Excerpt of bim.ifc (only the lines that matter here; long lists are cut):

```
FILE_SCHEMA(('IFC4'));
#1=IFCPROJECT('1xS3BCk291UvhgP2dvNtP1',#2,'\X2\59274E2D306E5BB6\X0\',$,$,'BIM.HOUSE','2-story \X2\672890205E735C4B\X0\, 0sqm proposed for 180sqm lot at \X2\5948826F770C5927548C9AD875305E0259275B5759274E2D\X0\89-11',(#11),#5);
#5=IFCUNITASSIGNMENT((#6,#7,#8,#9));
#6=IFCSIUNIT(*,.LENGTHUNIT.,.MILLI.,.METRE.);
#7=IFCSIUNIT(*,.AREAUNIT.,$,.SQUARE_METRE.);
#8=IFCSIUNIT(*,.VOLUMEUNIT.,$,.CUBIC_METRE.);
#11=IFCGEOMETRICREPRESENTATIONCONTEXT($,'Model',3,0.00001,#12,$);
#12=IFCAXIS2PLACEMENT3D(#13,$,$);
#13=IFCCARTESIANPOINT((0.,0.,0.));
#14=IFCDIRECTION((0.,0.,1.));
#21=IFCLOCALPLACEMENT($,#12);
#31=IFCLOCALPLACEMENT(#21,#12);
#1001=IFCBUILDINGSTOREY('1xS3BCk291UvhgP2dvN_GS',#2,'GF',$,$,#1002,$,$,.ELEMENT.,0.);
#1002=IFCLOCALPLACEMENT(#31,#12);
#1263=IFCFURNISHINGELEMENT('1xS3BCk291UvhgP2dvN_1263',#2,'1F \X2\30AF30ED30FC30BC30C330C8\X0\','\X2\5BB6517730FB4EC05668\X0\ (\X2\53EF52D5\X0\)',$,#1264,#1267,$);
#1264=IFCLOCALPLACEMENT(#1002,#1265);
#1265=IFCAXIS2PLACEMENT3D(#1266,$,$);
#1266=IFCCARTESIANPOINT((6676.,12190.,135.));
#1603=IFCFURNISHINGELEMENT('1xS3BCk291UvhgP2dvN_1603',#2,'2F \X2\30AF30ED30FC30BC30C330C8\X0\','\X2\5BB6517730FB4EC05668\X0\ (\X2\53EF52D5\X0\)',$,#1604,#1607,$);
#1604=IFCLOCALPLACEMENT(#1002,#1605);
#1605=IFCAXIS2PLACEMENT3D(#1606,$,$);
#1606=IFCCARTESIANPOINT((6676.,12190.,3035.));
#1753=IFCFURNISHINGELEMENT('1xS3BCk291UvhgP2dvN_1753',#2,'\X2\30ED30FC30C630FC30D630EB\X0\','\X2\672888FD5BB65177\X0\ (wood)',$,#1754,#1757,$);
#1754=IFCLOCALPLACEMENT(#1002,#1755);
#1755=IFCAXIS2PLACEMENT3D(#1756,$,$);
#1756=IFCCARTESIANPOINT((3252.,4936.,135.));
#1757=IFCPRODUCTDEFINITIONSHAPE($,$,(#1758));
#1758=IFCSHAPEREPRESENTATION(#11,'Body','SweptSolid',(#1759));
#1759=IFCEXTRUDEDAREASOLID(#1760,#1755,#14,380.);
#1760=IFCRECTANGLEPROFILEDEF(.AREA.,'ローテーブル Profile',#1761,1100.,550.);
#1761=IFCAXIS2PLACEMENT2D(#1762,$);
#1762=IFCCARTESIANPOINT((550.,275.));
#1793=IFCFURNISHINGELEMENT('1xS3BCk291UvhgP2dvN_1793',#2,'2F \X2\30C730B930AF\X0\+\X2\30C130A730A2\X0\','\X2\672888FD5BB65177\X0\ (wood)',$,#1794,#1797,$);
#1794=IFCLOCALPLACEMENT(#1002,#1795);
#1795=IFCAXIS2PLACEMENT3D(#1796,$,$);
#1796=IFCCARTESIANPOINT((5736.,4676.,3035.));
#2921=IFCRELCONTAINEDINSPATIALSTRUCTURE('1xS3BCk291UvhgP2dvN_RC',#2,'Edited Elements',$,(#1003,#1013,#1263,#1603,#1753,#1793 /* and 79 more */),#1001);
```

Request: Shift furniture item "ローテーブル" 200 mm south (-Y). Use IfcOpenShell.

```python
import ifcopenshell
import ifcopenshell.api.geometry
import ifcopenshell.util.placement

model = ifcopenshell.open("bim.ifc")

item = model.by_guid("1xS3BCk291UvhgP2dvN_1753")
matrix = ifcopenshell.util.placement.get_local_placement(item.ObjectPlacement)
matrix[1, 3] -= 200.0
ifcopenshell.api.geometry.edit_object_placement(model, product=item, matrix=matrix, is_si=False)

print(ifcopenshell.util.placement.get_local_placement(item.ObjectPlacement).round(3) + 0.0)

model.write("bim_updated.ifc")
```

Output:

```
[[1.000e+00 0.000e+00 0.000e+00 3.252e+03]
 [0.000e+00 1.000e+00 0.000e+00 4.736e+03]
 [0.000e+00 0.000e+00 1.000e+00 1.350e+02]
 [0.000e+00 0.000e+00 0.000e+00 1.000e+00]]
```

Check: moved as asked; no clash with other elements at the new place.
